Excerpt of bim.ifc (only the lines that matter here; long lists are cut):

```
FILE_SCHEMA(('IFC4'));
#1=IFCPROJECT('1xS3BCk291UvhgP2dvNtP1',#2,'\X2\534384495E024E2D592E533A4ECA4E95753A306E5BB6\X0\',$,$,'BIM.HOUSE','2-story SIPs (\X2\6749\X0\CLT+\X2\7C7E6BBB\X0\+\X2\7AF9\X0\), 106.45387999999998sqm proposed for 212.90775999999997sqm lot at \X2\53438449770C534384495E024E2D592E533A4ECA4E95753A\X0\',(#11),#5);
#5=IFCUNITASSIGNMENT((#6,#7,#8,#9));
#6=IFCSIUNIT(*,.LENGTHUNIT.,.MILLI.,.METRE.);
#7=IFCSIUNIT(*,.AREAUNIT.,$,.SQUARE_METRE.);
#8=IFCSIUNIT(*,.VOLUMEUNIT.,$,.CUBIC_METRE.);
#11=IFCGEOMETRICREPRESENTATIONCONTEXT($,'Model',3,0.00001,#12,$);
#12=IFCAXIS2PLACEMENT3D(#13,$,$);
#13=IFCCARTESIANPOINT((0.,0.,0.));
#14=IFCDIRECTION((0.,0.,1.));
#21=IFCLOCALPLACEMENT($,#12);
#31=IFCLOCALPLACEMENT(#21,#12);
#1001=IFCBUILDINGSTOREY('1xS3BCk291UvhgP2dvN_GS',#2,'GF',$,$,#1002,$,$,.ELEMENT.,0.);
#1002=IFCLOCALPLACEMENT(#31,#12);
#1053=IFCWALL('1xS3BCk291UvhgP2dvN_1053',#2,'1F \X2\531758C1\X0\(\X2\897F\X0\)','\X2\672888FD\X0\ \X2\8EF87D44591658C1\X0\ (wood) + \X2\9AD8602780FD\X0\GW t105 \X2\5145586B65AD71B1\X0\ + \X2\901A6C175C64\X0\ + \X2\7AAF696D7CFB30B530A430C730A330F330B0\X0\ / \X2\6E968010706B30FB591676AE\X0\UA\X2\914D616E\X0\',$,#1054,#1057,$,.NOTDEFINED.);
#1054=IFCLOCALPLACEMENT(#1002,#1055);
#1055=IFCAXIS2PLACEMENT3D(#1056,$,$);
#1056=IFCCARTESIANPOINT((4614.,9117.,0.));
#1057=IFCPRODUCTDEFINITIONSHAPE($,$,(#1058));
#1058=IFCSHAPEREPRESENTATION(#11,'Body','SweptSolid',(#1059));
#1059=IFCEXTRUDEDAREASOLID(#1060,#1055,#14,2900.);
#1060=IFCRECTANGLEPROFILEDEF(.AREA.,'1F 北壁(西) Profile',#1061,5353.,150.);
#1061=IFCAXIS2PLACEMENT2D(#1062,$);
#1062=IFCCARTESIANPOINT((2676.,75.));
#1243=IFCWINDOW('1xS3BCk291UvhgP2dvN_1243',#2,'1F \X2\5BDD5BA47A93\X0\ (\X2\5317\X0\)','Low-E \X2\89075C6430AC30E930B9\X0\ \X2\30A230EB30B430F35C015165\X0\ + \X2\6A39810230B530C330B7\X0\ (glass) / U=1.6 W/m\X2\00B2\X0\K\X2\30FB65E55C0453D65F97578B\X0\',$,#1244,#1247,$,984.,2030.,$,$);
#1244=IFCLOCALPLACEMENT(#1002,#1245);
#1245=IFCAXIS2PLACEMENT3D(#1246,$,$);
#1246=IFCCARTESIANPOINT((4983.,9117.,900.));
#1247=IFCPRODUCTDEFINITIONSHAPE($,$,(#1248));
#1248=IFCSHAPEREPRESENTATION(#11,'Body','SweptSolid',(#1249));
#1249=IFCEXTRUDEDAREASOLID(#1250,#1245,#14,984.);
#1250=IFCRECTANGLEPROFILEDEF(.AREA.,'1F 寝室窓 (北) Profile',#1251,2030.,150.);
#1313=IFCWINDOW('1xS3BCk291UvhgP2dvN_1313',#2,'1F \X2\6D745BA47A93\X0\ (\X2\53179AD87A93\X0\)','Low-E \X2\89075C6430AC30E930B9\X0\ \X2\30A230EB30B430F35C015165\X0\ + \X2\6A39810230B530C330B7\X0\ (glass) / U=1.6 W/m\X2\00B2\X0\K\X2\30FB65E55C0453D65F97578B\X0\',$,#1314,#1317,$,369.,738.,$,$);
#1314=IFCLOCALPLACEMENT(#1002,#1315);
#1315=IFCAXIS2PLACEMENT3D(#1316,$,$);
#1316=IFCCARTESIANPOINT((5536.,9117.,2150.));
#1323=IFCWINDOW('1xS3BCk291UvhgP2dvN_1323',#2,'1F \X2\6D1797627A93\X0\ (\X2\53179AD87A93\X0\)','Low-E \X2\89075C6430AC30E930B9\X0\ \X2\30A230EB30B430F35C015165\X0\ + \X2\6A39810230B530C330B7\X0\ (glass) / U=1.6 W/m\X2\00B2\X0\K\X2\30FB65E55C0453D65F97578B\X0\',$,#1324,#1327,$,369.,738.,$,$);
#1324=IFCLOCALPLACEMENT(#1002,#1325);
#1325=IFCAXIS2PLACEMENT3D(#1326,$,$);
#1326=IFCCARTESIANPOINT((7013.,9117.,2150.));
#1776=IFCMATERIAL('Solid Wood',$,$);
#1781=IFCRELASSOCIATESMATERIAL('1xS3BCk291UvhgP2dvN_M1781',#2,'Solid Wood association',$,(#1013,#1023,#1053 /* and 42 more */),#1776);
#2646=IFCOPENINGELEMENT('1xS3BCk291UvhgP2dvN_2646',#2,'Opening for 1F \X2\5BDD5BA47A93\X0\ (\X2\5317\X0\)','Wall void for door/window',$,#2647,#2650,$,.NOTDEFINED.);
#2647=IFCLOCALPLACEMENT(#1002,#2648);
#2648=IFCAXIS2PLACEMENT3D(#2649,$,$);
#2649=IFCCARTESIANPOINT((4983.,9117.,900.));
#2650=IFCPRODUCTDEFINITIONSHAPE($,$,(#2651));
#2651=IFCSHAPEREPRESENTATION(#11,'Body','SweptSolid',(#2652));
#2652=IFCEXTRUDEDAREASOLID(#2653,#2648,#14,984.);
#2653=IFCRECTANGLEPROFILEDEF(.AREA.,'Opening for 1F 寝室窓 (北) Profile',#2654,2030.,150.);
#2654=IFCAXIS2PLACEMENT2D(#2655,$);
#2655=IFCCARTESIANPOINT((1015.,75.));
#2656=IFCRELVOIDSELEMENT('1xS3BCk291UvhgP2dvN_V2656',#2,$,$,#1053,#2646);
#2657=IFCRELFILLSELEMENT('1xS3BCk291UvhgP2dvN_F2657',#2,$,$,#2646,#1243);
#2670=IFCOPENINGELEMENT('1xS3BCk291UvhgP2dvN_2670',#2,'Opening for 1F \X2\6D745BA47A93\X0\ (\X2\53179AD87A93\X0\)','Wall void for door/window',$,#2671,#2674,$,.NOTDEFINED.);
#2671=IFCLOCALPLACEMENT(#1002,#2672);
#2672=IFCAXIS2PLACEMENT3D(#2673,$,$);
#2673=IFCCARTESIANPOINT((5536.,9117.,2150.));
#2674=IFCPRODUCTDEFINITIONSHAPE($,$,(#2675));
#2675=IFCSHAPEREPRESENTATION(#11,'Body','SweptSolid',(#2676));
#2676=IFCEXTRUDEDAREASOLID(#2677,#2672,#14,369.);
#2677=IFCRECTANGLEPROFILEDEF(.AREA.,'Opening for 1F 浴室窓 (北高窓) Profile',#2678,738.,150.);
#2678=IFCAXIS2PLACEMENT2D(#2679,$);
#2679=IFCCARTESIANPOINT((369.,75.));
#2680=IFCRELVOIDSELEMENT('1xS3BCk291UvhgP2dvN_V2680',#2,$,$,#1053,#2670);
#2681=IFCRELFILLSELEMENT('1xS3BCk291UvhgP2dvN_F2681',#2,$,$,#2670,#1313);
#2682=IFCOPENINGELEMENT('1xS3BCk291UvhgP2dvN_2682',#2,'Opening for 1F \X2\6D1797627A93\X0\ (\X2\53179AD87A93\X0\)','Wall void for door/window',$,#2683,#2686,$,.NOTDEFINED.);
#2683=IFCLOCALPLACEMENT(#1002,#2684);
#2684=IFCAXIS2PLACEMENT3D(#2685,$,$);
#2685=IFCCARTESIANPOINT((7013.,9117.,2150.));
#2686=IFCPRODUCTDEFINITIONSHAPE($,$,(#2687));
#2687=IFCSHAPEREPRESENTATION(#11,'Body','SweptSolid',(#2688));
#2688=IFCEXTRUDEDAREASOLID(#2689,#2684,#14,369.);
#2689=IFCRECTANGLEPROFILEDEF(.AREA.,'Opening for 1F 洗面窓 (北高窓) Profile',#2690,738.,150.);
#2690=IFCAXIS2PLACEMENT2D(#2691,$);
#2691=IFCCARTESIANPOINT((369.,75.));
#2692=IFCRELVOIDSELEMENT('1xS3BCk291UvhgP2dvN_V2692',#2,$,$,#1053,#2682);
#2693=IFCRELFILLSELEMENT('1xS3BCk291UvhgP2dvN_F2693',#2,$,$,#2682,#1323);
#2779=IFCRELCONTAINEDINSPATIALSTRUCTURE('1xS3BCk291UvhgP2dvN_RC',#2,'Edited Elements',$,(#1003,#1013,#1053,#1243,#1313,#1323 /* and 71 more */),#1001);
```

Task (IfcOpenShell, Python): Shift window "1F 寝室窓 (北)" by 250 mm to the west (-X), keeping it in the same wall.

```python
import ifcopenshell
import ifcopenshell.api.geometry
import ifcopenshell.util.placement
import ifcopenshell.util.unit

model = ifcopenshell.open("bim.ifc")
unit_scale = ifcopenshell.util.unit.calculate_unit_scale(model)

window = model.by_guid("1xS3BCk291UvhgP2dvN_1243")
opening = window.FillsVoids[0].RelatingOpeningElement
wall = opening.VoidsElements[0].RelatingBuildingElement

wall_matrix = ifcopenshell.util.placement.get_local_placement(wall.ObjectPlacement)
shift = wall_matrix[:3, 0] * -0.25 / unit_scale
before = ifcopenshell.util.placement.get_local_placement(window.ObjectPlacement)[:3, 3].copy()

# The window is not placed relative to its opening, so move both.
for product in (opening, window):
    matrix = ifcopenshell.util.placement.get_local_placement(product.ObjectPlacement)
    matrix[:3, 3] += shift
    ifcopenshell.api.geometry.edit_object_placement(model, product=product, matrix=matrix, is_si=False)

after = ifcopenshell.util.placement.get_local_placement(window.ObjectPlacement)[:3, 3]
print("window moved by", (after - before).round(3) + 0.0)

model.write("bim_edited.ifc")
```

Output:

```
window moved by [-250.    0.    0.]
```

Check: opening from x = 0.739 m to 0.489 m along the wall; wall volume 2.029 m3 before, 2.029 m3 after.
